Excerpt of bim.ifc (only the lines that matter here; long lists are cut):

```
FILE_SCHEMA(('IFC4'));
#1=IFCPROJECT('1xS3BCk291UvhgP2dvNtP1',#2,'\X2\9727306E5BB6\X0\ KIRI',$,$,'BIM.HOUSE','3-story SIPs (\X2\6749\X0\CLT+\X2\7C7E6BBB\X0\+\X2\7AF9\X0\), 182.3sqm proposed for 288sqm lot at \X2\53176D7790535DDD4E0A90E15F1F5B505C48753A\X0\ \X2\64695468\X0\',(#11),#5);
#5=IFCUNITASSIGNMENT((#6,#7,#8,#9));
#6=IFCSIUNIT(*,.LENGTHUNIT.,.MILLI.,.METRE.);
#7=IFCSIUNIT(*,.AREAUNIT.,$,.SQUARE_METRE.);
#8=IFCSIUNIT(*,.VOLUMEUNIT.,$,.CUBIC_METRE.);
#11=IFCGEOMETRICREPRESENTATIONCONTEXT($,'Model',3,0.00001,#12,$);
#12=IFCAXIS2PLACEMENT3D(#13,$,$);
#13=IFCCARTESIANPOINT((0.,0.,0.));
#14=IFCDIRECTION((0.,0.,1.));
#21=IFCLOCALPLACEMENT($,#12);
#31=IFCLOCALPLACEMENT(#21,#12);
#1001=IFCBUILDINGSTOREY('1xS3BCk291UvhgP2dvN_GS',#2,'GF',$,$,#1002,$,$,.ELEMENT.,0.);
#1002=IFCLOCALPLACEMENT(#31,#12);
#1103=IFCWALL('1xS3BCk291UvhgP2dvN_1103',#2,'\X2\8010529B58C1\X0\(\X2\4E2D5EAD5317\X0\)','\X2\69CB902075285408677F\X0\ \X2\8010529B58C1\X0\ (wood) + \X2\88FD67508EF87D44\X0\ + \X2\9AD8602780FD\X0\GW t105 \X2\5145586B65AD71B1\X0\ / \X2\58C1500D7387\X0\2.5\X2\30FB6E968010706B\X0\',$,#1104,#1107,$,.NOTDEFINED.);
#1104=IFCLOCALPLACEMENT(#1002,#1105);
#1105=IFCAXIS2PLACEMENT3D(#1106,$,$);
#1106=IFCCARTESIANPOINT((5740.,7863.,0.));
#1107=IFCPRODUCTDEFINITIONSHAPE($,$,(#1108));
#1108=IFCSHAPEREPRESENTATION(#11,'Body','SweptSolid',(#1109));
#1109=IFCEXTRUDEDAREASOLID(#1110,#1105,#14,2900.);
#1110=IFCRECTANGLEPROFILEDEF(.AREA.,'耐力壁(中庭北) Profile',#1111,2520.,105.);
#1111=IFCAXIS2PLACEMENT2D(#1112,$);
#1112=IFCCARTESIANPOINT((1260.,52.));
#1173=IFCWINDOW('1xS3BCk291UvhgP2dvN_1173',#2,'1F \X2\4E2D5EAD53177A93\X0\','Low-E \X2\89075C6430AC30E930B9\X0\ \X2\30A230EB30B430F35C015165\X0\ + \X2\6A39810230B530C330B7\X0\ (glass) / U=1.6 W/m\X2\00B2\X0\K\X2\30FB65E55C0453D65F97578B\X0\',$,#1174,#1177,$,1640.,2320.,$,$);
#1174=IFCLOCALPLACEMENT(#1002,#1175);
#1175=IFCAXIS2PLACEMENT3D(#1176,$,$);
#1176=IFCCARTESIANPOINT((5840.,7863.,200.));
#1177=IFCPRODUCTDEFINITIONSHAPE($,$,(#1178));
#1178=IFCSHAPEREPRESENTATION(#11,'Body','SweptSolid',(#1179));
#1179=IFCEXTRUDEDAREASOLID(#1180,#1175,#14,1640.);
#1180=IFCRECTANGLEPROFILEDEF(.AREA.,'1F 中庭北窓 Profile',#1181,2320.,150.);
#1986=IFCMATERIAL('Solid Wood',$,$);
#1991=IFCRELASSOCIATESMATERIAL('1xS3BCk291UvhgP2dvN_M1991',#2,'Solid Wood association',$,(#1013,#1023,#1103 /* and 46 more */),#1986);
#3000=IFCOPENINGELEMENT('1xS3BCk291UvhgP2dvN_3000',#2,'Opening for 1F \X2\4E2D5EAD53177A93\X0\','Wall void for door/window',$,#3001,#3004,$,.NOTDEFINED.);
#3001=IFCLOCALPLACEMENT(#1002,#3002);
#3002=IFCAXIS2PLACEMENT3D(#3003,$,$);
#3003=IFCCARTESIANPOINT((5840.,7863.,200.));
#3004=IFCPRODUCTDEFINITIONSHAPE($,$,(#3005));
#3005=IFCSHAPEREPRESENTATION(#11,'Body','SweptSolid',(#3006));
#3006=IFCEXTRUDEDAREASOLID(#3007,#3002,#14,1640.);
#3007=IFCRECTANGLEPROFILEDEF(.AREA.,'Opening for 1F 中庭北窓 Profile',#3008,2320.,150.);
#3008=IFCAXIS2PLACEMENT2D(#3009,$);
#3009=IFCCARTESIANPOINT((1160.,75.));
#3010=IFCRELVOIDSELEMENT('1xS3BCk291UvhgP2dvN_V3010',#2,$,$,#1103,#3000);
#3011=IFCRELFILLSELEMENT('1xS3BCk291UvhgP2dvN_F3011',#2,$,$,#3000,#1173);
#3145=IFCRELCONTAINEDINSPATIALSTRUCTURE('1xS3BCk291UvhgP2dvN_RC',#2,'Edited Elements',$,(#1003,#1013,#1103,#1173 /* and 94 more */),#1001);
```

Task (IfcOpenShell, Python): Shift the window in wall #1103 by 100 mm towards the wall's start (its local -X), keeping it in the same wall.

```python
import ifcopenshell
import ifcopenshell.api.geometry
import ifcopenshell.util.placement
import ifcopenshell.util.unit

model = ifcopenshell.open("bim.ifc")
unit_scale = ifcopenshell.util.unit.calculate_unit_scale(model)

window = model.by_guid("1xS3BCk291UvhgP2dvN_1173")
opening = window.FillsVoids[0].RelatingOpeningElement
wall = opening.VoidsElements[0].RelatingBuildingElement

wall_matrix = ifcopenshell.util.placement.get_local_placement(wall.ObjectPlacement)
shift = wall_matrix[:3, 0] * -0.1 / unit_scale
before = ifcopenshell.util.placement.get_local_placement(window.ObjectPlacement)[:3, 3].copy()

# The window is not placed relative to its opening, so move both.
for product in (opening, window):
    matrix = ifcopenshell.util.placement.get_local_placement(product.ObjectPlacement)
    matrix[:3, 3] += shift
    ifcopenshell.api.geometry.edit_object_placement(model, product=product, matrix=matrix, is_si=False)

after = ifcopenshell.util.placement.get_local_placement(window.ObjectPlacement)[:3, 3]
print("window moved by", (after - before).round(3) + 0.0)

model.write("bim_edited.ifc")
```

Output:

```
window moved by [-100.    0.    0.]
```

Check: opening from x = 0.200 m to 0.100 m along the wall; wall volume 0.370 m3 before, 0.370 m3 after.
